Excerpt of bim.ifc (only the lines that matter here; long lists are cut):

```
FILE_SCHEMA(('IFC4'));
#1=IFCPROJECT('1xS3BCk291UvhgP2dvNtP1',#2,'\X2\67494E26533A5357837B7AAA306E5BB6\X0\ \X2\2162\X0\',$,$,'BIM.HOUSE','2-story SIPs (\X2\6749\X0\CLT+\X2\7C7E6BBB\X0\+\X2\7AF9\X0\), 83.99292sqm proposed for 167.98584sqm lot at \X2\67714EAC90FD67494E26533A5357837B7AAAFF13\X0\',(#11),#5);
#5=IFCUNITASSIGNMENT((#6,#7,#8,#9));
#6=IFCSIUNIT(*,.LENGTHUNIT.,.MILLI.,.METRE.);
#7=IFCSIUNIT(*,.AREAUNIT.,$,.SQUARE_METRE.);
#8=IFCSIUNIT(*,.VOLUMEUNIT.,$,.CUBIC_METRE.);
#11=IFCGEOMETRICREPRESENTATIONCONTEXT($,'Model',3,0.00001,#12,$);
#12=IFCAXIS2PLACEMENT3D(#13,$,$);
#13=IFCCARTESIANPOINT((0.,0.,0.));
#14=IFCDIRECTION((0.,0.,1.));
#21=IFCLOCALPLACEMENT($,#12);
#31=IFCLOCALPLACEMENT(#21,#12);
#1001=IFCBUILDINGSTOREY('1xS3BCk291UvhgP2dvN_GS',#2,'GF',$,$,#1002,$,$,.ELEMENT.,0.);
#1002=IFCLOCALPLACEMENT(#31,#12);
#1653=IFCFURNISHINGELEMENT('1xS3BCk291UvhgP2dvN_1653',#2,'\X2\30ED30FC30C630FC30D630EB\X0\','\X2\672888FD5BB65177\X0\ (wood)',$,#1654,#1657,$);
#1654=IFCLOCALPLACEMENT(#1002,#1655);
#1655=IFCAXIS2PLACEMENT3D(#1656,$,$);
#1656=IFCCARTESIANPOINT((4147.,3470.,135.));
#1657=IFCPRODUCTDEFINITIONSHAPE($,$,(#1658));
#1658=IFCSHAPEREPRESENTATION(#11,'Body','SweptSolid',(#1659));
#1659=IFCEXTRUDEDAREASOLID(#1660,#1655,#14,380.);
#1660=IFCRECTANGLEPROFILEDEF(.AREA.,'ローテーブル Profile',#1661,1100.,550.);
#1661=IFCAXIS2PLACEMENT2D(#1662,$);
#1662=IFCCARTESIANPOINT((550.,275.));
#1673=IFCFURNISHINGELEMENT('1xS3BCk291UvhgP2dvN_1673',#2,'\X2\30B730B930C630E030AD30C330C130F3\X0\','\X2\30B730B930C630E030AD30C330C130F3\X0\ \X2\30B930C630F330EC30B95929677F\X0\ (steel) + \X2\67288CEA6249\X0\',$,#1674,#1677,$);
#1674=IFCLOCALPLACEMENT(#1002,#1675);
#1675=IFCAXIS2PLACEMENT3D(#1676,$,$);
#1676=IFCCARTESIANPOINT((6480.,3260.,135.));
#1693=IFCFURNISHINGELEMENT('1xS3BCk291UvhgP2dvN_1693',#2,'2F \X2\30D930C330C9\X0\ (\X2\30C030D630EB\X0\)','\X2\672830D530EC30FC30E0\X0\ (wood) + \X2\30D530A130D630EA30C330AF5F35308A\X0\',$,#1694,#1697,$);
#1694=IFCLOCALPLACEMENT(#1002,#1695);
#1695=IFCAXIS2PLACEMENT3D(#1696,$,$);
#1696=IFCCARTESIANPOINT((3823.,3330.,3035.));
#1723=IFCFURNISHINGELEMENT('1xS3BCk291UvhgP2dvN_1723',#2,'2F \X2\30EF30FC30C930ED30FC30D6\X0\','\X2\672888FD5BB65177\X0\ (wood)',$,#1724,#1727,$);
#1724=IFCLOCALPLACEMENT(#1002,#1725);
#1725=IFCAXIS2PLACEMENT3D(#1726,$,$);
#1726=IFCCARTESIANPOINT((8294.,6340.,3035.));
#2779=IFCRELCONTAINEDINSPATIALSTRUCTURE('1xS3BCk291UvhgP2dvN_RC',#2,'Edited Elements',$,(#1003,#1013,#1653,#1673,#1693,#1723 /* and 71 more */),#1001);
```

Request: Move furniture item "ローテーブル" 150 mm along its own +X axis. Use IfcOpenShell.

```python
import ifcopenshell
import ifcopenshell.api.geometry
import ifcopenshell.util.placement

model = ifcopenshell.open("bim.ifc")

item = model.by_id(1653)
matrix = ifcopenshell.util.placement.get_local_placement(item.ObjectPlacement)
matrix[:3, 3] += matrix[:3, 0] * 150.0
ifcopenshell.api.geometry.edit_object_placement(model, product=item, matrix=matrix, is_si=False)

print(ifcopenshell.util.placement.get_local_placement(item.ObjectPlacement).round(3) + 0.0)

model.write("bim_rev.ifc")
```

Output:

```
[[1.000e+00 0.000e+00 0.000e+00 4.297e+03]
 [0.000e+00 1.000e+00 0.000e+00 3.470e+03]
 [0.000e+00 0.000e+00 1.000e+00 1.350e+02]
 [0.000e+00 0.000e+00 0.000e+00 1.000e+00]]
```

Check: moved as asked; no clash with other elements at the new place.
